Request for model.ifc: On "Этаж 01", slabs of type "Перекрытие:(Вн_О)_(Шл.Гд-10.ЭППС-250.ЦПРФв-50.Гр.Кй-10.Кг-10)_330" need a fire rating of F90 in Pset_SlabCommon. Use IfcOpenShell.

First a look at what the model holds.

```python
import ifcopenshell
import ifcopenshell.util.element

model = ifcopenshell.open("model.ifc")
print(model.schema)
storey = next(s for s in model.by_type("IfcBuildingStorey") if s.Name == "Этаж 01")
slabs = [e for e in ifcopenshell.util.element.get_decomposition(storey) if e.is_a("IfcSlab")]
seen = {}
for e in slabs:
    element_type = ifcopenshell.util.element.get_type(e)
    key = (element_type.Name if element_type != e and element_type else None, ifcopenshell.util.element.get_pset(e, "Pset_SlabCommon", "FireRating"))
    seen[key] = seen.get(key, 0) + 1
for (name, value), count in sorted(seen.items(), key=str):
    print(count, "x", name, "|", value)
```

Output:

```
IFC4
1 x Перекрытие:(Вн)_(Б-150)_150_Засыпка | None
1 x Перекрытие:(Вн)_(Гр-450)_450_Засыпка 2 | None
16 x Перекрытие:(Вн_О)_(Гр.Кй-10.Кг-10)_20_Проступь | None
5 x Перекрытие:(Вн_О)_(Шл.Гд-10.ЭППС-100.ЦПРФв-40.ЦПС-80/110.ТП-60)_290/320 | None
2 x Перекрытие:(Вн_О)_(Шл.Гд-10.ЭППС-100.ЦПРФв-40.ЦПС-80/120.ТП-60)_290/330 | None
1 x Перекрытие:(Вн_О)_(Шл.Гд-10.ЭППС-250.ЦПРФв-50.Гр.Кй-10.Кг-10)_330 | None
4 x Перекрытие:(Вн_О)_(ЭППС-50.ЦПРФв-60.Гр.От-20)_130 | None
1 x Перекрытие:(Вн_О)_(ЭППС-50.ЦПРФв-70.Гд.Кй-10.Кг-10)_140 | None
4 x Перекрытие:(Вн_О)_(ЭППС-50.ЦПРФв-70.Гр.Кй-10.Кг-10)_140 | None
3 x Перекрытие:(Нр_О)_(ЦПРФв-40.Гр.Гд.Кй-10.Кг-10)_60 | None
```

```python
import ifcopenshell
import ifcopenshell.api.pset
import ifcopenshell.util.element

model = ifcopenshell.open("model.ifc")

storey = next(s for s in model.by_type("IfcBuildingStorey") if s.Name == "Этаж 01")
slabs = [e for e in ifcopenshell.util.element.get_decomposition(storey) if e.is_a("IfcSlab")]

count = 0
for e in slabs:
    element_type = ifcopenshell.util.element.get_type(e)
    if element_type in (None, e) or element_type.Name != "Перекрытие:(Вн_О)_(Шл.Гд-10.ЭППС-250.ЦПРФв-50.Гр.Кй-10.Кг-10)_330":
        continue
    # add_pset returns the element's existing set when there is one.
    pset = ifcopenshell.api.pset.add_pset(model, product=e, name="Pset_SlabCommon")
    ifcopenshell.api.pset.edit_pset(model, pset=pset, properties={"FireRating": "F90"})
    count += 1

print(count, "slabs updated")

model.write("model_rev.ifc")
```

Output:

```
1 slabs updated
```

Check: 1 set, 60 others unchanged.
